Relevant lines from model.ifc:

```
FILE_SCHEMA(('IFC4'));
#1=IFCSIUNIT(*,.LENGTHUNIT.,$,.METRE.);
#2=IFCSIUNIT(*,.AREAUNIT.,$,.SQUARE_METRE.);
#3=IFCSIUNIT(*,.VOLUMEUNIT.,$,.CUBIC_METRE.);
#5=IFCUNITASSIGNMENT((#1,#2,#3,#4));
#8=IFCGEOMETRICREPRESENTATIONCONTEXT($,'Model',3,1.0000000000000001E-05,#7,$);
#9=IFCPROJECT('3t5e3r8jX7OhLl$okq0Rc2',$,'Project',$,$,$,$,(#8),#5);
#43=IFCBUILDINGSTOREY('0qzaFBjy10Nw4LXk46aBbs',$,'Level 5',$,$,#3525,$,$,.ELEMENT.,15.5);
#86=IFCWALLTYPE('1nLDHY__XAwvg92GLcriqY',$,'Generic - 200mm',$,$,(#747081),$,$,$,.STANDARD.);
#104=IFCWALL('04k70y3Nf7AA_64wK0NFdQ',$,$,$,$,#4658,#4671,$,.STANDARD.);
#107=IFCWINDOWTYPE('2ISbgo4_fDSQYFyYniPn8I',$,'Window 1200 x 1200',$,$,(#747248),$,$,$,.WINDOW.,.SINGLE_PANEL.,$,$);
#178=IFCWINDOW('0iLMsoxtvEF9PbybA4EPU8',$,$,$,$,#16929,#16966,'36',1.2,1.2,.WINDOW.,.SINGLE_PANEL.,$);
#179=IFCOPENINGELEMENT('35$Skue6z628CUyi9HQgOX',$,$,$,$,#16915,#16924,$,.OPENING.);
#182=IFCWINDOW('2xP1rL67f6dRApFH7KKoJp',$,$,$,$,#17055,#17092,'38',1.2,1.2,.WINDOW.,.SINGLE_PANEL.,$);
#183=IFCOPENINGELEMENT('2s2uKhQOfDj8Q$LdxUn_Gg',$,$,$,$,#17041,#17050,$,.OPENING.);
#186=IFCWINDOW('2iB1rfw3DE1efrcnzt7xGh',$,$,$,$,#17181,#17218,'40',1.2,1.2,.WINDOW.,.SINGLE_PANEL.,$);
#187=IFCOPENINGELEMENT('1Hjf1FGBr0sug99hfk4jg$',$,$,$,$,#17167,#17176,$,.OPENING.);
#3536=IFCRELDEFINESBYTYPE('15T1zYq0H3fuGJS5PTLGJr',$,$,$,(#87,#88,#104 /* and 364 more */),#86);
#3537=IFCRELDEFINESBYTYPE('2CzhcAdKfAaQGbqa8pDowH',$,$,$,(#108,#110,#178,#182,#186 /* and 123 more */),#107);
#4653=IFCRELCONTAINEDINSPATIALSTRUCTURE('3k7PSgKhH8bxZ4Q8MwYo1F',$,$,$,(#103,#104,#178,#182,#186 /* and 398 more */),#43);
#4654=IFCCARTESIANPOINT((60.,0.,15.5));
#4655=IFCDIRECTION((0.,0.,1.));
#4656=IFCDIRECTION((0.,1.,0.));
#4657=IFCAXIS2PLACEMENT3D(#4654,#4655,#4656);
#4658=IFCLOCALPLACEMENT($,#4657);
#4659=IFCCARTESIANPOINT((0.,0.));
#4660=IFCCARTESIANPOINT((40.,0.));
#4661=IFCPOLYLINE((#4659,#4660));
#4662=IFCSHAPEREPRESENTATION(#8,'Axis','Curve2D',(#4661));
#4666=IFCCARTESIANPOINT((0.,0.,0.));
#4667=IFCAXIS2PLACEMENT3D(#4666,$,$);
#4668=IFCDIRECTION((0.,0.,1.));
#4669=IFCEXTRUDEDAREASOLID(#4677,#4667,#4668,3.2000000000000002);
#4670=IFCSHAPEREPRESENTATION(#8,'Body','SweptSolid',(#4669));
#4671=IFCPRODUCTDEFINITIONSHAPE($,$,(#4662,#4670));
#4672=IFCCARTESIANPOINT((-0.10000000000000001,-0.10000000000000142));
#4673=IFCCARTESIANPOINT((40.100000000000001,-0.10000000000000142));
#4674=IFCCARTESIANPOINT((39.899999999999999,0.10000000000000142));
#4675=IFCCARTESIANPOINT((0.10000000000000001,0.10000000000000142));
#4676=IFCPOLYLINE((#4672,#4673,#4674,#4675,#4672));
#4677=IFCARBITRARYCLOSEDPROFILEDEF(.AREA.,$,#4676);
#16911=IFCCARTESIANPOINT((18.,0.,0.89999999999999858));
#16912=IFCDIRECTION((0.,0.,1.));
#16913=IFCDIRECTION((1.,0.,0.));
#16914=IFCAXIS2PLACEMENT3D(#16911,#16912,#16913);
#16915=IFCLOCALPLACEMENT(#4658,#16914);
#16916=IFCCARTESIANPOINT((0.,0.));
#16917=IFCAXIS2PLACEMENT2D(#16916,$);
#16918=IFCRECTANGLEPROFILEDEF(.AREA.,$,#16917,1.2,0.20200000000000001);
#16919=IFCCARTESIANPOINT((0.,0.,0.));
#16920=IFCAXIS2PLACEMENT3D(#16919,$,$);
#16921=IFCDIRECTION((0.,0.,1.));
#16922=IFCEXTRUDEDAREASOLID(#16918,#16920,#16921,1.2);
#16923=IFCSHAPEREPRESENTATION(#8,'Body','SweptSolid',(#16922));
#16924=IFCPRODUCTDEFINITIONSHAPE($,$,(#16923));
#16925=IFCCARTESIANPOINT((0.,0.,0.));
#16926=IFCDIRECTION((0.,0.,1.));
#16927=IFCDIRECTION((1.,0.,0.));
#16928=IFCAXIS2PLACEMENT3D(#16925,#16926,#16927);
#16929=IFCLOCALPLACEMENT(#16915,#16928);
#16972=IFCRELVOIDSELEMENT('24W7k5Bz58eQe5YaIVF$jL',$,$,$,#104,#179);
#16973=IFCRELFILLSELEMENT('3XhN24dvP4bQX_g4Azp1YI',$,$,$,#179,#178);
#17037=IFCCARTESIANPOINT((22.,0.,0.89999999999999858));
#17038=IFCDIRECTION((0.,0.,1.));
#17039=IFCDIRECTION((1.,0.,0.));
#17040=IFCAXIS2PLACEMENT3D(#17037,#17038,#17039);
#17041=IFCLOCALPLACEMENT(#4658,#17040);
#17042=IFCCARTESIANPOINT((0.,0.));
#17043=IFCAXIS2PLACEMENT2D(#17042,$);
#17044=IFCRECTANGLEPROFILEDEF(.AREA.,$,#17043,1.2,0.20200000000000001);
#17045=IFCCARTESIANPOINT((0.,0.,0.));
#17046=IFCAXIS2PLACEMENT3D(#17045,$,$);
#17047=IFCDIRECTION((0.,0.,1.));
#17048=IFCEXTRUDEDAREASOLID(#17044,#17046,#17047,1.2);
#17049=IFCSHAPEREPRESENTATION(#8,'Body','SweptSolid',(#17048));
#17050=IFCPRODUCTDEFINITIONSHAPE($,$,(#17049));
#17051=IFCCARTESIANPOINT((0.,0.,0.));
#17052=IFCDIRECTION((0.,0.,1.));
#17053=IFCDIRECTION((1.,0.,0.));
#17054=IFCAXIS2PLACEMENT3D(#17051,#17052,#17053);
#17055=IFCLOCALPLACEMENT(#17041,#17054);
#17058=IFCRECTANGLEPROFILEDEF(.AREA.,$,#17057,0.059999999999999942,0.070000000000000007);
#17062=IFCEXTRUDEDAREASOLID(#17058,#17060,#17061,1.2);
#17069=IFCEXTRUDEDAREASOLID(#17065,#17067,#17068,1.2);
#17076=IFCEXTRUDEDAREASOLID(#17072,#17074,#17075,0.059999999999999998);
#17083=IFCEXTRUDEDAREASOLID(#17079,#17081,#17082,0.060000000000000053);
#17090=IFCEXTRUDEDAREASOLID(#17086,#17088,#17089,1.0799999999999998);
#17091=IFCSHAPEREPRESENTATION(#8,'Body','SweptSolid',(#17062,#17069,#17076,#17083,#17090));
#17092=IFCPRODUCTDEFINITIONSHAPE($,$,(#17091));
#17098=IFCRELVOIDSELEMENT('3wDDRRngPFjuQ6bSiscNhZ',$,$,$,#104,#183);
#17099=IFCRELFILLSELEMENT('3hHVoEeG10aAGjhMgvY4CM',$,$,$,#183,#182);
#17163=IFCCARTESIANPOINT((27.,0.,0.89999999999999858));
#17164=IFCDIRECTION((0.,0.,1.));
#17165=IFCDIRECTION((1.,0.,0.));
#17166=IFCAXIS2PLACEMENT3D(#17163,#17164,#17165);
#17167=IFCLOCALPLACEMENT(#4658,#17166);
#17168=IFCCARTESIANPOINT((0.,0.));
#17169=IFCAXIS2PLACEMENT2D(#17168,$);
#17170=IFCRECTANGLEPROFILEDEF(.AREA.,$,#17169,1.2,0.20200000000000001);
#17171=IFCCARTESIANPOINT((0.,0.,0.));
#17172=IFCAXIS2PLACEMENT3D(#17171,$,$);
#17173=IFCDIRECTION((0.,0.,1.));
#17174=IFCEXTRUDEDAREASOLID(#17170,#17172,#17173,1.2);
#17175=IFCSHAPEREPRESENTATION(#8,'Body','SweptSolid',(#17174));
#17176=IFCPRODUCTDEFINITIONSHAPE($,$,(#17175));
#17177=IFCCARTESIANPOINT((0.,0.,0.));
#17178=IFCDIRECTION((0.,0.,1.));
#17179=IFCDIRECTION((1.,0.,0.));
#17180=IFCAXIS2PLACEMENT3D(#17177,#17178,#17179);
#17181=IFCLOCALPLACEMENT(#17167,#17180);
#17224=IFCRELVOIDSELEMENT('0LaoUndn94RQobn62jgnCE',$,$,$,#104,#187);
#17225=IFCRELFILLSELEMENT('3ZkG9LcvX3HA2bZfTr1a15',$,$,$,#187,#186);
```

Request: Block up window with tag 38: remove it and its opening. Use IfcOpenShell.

```python
import ifcopenshell
import ifcopenshell.api.feature
import ifcopenshell.api.root
import ifcopenshell.geom
import ifcopenshell.util.shape

model = ifcopenshell.open("model.ifc")
settings = ifcopenshell.geom.settings()


def volume(element):
    """Net volume in cubic metres, openings subtracted."""
    shape = ifcopenshell.geom.create_shape(settings, element)
    return ifcopenshell.util.shape.get_volume(shape.geometry)


window = model.by_guid("2xP1rL67f6dRApFH7KKoJp")
opening = window.FillsVoids[0].RelatingOpeningElement
wall = opening.VoidsElements[0].RelatingBuildingElement
before = volume(wall)

ifcopenshell.api.root.remove_product(model, product=window)
ifcopenshell.api.feature.remove_feature(model, feature=opening)

after = volume(wall)

print(f"wall volume {before:.3f} -> {after:.3f} m3")

model.write("model-out.ifc")
```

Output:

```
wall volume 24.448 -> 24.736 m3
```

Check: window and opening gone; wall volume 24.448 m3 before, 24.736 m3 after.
